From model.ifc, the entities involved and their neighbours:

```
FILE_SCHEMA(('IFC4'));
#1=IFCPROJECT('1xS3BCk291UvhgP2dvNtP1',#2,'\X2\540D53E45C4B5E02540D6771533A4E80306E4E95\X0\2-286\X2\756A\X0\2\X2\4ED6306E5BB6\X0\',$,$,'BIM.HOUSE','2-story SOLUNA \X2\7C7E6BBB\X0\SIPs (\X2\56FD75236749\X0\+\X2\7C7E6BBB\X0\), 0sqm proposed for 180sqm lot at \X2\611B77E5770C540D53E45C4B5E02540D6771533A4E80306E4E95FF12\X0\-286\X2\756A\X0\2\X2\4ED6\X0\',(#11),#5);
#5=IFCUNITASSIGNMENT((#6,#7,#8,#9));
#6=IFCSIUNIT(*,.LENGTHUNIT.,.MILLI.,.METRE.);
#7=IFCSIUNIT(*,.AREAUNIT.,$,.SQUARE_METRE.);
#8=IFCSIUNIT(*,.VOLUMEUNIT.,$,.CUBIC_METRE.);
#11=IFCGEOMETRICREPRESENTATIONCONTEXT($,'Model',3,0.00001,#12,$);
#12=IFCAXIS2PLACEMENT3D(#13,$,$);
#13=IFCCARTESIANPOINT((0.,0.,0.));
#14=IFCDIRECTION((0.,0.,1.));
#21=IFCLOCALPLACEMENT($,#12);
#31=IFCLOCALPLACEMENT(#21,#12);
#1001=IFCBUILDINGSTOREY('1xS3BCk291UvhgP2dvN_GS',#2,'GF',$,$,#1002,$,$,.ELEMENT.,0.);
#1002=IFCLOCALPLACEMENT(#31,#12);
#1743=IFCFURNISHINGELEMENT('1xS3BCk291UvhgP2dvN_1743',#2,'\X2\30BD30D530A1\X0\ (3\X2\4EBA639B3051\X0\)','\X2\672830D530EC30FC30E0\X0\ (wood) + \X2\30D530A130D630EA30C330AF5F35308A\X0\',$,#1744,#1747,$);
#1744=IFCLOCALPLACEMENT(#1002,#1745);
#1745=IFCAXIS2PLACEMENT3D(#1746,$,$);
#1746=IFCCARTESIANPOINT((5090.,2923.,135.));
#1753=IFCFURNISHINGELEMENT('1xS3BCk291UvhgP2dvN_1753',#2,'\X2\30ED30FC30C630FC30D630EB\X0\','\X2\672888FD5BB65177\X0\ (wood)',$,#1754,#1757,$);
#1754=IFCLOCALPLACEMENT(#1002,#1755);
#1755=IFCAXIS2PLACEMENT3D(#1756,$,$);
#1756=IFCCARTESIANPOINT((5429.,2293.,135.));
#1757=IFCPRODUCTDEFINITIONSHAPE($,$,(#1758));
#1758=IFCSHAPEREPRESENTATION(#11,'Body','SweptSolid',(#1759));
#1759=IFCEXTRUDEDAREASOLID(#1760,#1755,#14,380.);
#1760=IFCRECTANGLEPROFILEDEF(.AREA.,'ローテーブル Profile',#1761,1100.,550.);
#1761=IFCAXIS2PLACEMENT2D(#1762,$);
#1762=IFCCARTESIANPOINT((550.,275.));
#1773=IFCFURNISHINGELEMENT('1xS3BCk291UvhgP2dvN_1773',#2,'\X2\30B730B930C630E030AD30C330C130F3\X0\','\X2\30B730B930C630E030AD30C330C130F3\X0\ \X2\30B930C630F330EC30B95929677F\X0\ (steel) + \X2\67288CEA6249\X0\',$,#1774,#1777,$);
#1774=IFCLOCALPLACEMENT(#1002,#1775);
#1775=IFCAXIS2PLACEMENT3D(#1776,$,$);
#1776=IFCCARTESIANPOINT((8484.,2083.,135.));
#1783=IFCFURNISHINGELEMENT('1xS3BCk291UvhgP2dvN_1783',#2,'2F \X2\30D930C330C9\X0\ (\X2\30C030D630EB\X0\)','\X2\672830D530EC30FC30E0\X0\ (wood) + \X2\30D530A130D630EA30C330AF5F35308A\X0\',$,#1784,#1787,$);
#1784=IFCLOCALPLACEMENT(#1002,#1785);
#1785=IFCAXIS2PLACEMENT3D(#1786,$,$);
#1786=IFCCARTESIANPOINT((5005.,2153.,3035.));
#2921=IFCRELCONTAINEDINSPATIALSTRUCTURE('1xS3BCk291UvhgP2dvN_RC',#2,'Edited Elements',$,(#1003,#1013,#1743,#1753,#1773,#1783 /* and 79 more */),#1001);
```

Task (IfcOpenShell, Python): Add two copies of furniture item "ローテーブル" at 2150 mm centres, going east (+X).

```python
import numpy as np
import ifcopenshell
import ifcopenshell.api.geometry
import ifcopenshell.api.root
import ifcopenshell.util.element
import ifcopenshell.util.placement

model = ifcopenshell.open("model.ifc")


def reuse_history(source, copy):
    """copy_class also copies each property set's owner history, people and application; keep the originals."""
    for rel in copy.IsDefinedBy:
        if rel.is_a("IfcRelDefinesByProperties") and (history := rel.RelatingPropertyDefinition.OwnerHistory):
            rel.RelatingPropertyDefinition.OwnerHistory = source.OwnerHistory
            ifcopenshell.util.element.remove_deep2(model, history)


source = model.by_guid("1xS3BCk291UvhgP2dvN_1753")
base = ifcopenshell.util.placement.get_local_placement(source.ObjectPlacement)
step = np.array([1.0, 0.0, 0.0]) * 2150.0

for i in range(1, 3):
    copy = ifcopenshell.api.root.copy_class(model, product=source)
    copy.Representation = ifcopenshell.util.element.copy_deep(
        model, source.Representation, exclude=["IfcGeometricRepresentationContext", "IfcRepresentationMap"]
    )
    reuse_history(source, copy)
    matrix = base.copy()
    matrix[:3, 3] += i * step
    print("added at", matrix[:3, 3].round(3) + 0.0)
    ifcopenshell.api.geometry.edit_object_placement(model, product=copy, matrix=matrix, is_si=False)

model.write("model_v2.ifc")
```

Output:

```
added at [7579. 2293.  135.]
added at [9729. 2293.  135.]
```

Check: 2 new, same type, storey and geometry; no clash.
